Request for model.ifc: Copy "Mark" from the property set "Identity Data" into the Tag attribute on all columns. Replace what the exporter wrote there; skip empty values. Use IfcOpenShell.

First a look at what the model holds.

```python
import ifcopenshell
import ifcopenshell.util.element

model = ifcopenshell.open("model.ifc")
print(model.schema)
columns = model.by_type("IfcColumn")
print(len(columns), "columns")
for e in columns[:8]:
    source = ifcopenshell.util.element.get_pset(e, "Identity Data", "Mark")
    target = e.Tag
    print(e.id(), repr(source), repr(target), sep=" | ")
```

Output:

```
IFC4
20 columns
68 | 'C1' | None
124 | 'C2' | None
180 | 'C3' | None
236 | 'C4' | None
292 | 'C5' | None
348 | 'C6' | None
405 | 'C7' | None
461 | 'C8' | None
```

```python
import ifcopenshell
import ifcopenshell.util.element

model = ifcopenshell.open("model.ifc")

count = 0
for e in model.by_type("IfcColumn"):
    value = ifcopenshell.util.element.get_pset(e, "Identity Data", "Mark")
    current = e.Tag
    if not value or not value.strip() or current == value:
        continue
    e.Tag = value
    count += 1

print(count, "columns updated")

model.write("model_v2.ifc")
```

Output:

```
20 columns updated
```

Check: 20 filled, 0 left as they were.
